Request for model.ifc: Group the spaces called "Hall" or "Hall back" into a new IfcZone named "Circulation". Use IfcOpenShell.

First a look at what the model holds.

```python
import ifcopenshell

model = ifcopenshell.open("model.ifc")
print(model.schema)
seen = {}
for space in model.by_type("IfcSpace"):
    seen[space.LongName] = seen.get(space.LongName, 0) + 1
for name, count in sorted(seen.items(), key=str):
    print(count, "x", name)
print("zones:", [z.Name for z in model.by_type("IfcZone")][:20])
```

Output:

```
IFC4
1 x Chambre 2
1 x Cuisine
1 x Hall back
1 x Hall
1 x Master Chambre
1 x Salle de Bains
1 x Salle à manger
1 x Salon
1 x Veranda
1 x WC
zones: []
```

```python
import ifcopenshell
import ifcopenshell.api.group
import ifcopenshell.api.root

model = ifcopenshell.open("model.ifc")

names = {"Hall", "Hall back"}
spaces = [s for s in model.by_type("IfcSpace") if s.LongName in names]

zone = ifcopenshell.api.root.create_entity(model, ifc_class="IfcZone", name="Circulation")
ifcopenshell.api.group.assign_group(model, products=spaces, group=zone)
print(len(spaces), "spaces in", zone.Name)

model.write("model_edited.ifc")
```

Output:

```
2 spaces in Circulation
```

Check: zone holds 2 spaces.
